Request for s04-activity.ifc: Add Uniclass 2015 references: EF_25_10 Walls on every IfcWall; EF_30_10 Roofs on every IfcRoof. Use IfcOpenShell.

First a look at what the model holds.

```python
import ifcopenshell

model = ifcopenshell.open("s04-activity.ifc")
print(model.schema)
print("classifications:", [c.Name for c in model.by_type("IfcClassification")])
for ifc_class in ("IfcDoor", "IfcRoof", "IfcStair", "IfcWall", "IfcWindow"):
    print(ifc_class, len(model.by_type(ifc_class)))
```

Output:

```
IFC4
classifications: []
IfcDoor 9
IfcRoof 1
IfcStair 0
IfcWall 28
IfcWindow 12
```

```python
import ifcopenshell
import ifcopenshell.api.classification

model = ifcopenshell.open("s04-activity.ifc")

system = ifcopenshell.api.classification.add_classification(model, classification="Uniclass 2015")

codes = {
    "IfcWall": ("EF_25_10", "Walls"),
    "IfcRoof": ("EF_30_10", "Roofs"),
}
for ifc_class, (code, name) in codes.items():
    products = model.by_type(ifc_class)
    ifcopenshell.api.classification.add_reference(
        model, products=products, classification=system, identification=code, name=name
    )
    print(code, len(products))

model.write("s04-activity_v2.ifc")
```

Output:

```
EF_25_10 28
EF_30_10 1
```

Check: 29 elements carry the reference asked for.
